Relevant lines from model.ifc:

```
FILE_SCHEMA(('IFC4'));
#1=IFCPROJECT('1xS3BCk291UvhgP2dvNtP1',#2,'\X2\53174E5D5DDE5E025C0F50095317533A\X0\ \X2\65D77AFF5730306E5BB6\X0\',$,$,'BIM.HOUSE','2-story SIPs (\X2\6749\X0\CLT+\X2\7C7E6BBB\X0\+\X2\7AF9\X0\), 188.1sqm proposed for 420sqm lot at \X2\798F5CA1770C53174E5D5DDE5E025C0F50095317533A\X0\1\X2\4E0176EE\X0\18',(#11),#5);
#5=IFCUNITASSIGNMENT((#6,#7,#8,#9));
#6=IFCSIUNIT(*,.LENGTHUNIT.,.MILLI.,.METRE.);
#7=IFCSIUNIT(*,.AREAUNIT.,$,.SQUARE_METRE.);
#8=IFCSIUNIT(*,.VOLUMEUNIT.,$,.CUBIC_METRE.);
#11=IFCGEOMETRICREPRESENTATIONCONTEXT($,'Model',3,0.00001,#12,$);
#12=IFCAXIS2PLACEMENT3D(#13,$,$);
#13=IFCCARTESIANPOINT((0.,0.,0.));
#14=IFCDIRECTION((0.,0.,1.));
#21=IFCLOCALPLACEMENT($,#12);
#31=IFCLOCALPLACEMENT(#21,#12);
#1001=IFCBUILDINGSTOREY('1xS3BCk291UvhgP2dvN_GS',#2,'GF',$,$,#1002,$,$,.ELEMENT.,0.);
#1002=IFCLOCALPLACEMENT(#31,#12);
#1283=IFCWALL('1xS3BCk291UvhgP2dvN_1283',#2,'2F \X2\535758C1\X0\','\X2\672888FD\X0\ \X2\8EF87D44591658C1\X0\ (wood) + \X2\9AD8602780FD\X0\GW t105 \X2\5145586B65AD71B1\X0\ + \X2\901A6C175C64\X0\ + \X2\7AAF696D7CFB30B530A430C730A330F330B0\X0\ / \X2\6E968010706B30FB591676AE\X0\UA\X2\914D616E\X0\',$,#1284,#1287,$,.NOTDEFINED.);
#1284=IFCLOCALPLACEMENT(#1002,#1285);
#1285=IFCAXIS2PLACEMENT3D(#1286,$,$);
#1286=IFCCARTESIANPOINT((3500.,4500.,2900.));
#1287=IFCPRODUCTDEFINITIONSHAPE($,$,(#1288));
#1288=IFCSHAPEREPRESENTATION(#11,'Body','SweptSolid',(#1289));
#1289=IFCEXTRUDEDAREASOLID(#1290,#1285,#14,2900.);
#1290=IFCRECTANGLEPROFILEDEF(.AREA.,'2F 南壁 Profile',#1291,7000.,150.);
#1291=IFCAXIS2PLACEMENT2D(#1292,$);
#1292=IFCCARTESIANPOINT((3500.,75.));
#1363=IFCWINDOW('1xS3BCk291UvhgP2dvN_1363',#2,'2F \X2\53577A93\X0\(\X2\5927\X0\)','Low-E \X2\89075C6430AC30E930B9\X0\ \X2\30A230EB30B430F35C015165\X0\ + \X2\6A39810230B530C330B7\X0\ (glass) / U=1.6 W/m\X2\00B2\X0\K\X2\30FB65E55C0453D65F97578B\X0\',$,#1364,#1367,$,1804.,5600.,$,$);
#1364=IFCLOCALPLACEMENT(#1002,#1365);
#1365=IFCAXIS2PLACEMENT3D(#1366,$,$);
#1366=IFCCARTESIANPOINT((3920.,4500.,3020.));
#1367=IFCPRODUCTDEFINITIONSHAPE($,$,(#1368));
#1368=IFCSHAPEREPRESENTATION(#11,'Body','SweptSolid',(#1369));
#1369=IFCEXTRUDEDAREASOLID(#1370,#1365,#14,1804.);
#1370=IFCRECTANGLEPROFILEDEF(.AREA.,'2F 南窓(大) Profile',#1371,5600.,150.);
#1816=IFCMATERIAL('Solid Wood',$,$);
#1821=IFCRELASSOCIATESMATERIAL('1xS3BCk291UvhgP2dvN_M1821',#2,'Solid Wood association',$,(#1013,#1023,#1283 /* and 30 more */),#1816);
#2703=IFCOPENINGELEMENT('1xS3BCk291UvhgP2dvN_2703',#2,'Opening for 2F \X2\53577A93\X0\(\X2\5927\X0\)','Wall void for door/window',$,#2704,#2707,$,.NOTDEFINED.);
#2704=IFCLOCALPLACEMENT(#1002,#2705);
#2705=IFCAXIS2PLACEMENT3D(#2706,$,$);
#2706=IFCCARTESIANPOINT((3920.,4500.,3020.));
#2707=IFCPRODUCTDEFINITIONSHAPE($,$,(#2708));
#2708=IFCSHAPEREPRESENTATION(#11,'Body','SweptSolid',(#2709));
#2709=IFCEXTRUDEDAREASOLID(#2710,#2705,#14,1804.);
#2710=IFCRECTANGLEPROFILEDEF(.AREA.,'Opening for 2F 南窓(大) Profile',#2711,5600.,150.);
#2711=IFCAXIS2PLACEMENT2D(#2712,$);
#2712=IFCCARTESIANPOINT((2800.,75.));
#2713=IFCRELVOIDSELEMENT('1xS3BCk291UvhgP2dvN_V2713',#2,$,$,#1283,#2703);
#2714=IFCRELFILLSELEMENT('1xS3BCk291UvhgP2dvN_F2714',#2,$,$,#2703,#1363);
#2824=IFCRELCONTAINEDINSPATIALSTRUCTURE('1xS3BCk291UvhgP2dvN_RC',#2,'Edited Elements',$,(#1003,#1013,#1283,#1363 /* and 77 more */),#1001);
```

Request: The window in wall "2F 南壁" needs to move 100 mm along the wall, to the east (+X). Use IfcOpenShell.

```python
import ifcopenshell
import ifcopenshell.api.geometry
import ifcopenshell.util.placement

model = ifcopenshell.open("model.ifc")

window = model.by_id(1363)
opening = window.FillsVoids[0].RelatingOpeningElement
wall = opening.VoidsElements[0].RelatingBuildingElement

wall_matrix = ifcopenshell.util.placement.get_local_placement(wall.ObjectPlacement)
shift = wall_matrix[:3, 0] * 100.0
before = ifcopenshell.util.placement.get_local_placement(window.ObjectPlacement)[:3, 3].copy()

# The window is not placed relative to its opening, so move both.
for product in (opening, window):
    matrix = ifcopenshell.util.placement.get_local_placement(product.ObjectPlacement)
    matrix[:3, 3] += shift
    ifcopenshell.api.geometry.edit_object_placement(model, product=product, matrix=matrix, is_si=False)

after = ifcopenshell.util.placement.get_local_placement(window.ObjectPlacement)[:3, 3]
print("window moved by", (after - before).round(3) + 0.0)

model.write("model_rev.ifc")
```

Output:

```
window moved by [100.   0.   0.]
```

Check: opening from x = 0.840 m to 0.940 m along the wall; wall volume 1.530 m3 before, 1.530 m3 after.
